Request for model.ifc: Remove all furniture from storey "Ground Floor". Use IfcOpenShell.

First a look at what the model holds.

```python
import ifcopenshell
import ifcopenshell.util.element

model = ifcopenshell.open("model.ifc")
print(model.schema)
storey = next(s for s in model.by_type("IfcBuildingStorey") if s.Name == "Ground Floor")
furniture = [e for e in ifcopenshell.util.element.get_decomposition(storey) if e.is_a("IfcFurnishingElement")]
seen = {}
for e in furniture:
    element_type = ifcopenshell.util.element.get_type(e)
    name = element_type.Name if element_type not in (None, e) else None
    seen[name] = seen.get(name, 0) + 1
for name, count in sorted(seen.items(), key=str):
    print(count, "x", name)
```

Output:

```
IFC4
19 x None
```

```python
import ifcopenshell
import ifcopenshell.api.root
import ifcopenshell.util.element

model = ifcopenshell.open("model.ifc")

storey = next(s for s in model.by_type("IfcBuildingStorey") if s.Name == "Ground Floor")
furniture = [e for e in ifcopenshell.util.element.get_decomposition(storey) if e.is_a("IfcFurnishingElement")]

for e in furniture:
    ifcopenshell.api.root.remove_product(model, product=e)
print(len(furniture), "removed")

model.write("model_updated.ifc")
```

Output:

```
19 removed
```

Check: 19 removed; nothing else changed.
